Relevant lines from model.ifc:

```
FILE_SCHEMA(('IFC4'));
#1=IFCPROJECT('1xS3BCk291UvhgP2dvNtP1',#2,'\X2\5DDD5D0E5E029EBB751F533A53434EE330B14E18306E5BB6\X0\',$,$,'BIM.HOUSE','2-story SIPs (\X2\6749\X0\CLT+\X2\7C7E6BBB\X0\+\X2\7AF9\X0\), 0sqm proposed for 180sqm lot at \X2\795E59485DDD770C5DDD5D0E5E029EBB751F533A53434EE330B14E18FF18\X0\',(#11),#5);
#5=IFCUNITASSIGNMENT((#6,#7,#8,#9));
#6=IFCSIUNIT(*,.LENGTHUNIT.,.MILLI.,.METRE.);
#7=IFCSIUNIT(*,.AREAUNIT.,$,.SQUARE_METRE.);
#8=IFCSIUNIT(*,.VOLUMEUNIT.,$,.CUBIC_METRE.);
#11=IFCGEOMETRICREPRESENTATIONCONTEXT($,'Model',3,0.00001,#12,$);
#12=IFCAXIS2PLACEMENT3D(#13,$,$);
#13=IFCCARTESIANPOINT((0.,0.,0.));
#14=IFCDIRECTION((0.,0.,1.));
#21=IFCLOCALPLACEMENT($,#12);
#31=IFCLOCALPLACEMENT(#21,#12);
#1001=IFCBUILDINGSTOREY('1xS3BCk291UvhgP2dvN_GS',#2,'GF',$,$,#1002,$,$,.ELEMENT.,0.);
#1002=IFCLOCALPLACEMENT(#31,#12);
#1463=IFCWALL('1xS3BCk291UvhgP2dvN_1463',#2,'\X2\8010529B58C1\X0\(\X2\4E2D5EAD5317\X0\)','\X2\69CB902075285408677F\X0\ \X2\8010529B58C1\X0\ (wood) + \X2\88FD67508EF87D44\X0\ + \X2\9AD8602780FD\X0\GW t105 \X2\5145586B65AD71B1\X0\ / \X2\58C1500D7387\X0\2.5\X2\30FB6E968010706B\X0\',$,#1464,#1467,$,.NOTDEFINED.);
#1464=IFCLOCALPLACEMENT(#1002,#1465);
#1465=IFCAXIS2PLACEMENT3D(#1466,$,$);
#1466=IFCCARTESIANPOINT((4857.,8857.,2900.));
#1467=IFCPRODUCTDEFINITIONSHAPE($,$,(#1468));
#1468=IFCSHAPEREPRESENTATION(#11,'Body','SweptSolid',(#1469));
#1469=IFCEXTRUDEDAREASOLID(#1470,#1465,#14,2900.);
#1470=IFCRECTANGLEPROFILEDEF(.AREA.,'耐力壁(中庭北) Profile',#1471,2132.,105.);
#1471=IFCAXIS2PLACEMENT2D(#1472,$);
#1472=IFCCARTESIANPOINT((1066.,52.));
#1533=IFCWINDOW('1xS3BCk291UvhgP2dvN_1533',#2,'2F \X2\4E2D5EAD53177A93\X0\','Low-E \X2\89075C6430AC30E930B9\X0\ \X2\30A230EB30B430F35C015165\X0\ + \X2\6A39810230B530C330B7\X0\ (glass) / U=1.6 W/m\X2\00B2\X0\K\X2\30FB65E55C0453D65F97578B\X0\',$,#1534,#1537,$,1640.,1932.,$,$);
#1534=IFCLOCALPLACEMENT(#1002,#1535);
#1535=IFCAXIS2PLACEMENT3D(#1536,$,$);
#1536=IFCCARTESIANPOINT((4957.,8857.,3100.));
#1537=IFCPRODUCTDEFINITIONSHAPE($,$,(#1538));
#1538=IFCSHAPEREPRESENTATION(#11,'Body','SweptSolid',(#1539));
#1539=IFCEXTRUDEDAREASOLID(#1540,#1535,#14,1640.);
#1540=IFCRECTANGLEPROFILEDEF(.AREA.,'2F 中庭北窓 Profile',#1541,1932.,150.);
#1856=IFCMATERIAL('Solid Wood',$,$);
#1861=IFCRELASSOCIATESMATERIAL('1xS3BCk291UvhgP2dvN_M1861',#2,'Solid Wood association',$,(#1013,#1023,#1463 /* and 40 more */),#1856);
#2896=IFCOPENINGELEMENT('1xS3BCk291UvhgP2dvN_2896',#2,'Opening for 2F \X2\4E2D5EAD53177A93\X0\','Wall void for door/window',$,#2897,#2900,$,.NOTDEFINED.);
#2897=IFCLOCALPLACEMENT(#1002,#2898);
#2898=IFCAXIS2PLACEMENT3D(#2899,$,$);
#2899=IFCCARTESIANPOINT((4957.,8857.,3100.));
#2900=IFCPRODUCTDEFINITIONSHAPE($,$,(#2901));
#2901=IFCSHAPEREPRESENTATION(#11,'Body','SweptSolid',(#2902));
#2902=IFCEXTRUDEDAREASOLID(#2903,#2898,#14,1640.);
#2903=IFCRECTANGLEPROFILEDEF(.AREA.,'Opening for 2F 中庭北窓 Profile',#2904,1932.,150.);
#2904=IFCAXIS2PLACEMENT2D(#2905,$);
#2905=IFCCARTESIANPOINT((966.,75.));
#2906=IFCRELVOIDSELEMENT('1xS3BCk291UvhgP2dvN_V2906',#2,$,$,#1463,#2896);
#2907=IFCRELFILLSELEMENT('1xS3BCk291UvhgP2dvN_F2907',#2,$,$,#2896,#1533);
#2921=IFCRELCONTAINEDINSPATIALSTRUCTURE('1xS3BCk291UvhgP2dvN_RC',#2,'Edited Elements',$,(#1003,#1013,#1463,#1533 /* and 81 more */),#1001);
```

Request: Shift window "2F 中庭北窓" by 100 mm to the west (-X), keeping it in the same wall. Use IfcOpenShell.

```python
import ifcopenshell
import ifcopenshell.api.geometry
import ifcopenshell.util.placement
import ifcopenshell.util.unit

model = ifcopenshell.open("model.ifc")
unit_scale = ifcopenshell.util.unit.calculate_unit_scale(model)

window = model.by_guid("1xS3BCk291UvhgP2dvN_1533")
opening = window.FillsVoids[0].RelatingOpeningElement
wall = opening.VoidsElements[0].RelatingBuildingElement

wall_matrix = ifcopenshell.util.placement.get_local_placement(wall.ObjectPlacement)
shift = wall_matrix[:3, 0] * -0.1 / unit_scale
before = ifcopenshell.util.placement.get_local_placement(window.ObjectPlacement)[:3, 3].copy()

# The window is not placed relative to its opening, so move both.
for product in (opening, window):
    matrix = ifcopenshell.util.placement.get_local_placement(product.ObjectPlacement)
    matrix[:3, 3] += shift
    ifcopenshell.api.geometry.edit_object_placement(model, product=product, matrix=matrix, is_si=False)

after = ifcopenshell.util.placement.get_local_placement(window.ObjectPlacement)[:3, 3]
print("window moved by", (after - before).round(3) + 0.0)

model.write("model_v2.ifc")
```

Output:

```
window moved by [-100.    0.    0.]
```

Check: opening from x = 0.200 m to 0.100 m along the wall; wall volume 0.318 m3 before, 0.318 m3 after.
